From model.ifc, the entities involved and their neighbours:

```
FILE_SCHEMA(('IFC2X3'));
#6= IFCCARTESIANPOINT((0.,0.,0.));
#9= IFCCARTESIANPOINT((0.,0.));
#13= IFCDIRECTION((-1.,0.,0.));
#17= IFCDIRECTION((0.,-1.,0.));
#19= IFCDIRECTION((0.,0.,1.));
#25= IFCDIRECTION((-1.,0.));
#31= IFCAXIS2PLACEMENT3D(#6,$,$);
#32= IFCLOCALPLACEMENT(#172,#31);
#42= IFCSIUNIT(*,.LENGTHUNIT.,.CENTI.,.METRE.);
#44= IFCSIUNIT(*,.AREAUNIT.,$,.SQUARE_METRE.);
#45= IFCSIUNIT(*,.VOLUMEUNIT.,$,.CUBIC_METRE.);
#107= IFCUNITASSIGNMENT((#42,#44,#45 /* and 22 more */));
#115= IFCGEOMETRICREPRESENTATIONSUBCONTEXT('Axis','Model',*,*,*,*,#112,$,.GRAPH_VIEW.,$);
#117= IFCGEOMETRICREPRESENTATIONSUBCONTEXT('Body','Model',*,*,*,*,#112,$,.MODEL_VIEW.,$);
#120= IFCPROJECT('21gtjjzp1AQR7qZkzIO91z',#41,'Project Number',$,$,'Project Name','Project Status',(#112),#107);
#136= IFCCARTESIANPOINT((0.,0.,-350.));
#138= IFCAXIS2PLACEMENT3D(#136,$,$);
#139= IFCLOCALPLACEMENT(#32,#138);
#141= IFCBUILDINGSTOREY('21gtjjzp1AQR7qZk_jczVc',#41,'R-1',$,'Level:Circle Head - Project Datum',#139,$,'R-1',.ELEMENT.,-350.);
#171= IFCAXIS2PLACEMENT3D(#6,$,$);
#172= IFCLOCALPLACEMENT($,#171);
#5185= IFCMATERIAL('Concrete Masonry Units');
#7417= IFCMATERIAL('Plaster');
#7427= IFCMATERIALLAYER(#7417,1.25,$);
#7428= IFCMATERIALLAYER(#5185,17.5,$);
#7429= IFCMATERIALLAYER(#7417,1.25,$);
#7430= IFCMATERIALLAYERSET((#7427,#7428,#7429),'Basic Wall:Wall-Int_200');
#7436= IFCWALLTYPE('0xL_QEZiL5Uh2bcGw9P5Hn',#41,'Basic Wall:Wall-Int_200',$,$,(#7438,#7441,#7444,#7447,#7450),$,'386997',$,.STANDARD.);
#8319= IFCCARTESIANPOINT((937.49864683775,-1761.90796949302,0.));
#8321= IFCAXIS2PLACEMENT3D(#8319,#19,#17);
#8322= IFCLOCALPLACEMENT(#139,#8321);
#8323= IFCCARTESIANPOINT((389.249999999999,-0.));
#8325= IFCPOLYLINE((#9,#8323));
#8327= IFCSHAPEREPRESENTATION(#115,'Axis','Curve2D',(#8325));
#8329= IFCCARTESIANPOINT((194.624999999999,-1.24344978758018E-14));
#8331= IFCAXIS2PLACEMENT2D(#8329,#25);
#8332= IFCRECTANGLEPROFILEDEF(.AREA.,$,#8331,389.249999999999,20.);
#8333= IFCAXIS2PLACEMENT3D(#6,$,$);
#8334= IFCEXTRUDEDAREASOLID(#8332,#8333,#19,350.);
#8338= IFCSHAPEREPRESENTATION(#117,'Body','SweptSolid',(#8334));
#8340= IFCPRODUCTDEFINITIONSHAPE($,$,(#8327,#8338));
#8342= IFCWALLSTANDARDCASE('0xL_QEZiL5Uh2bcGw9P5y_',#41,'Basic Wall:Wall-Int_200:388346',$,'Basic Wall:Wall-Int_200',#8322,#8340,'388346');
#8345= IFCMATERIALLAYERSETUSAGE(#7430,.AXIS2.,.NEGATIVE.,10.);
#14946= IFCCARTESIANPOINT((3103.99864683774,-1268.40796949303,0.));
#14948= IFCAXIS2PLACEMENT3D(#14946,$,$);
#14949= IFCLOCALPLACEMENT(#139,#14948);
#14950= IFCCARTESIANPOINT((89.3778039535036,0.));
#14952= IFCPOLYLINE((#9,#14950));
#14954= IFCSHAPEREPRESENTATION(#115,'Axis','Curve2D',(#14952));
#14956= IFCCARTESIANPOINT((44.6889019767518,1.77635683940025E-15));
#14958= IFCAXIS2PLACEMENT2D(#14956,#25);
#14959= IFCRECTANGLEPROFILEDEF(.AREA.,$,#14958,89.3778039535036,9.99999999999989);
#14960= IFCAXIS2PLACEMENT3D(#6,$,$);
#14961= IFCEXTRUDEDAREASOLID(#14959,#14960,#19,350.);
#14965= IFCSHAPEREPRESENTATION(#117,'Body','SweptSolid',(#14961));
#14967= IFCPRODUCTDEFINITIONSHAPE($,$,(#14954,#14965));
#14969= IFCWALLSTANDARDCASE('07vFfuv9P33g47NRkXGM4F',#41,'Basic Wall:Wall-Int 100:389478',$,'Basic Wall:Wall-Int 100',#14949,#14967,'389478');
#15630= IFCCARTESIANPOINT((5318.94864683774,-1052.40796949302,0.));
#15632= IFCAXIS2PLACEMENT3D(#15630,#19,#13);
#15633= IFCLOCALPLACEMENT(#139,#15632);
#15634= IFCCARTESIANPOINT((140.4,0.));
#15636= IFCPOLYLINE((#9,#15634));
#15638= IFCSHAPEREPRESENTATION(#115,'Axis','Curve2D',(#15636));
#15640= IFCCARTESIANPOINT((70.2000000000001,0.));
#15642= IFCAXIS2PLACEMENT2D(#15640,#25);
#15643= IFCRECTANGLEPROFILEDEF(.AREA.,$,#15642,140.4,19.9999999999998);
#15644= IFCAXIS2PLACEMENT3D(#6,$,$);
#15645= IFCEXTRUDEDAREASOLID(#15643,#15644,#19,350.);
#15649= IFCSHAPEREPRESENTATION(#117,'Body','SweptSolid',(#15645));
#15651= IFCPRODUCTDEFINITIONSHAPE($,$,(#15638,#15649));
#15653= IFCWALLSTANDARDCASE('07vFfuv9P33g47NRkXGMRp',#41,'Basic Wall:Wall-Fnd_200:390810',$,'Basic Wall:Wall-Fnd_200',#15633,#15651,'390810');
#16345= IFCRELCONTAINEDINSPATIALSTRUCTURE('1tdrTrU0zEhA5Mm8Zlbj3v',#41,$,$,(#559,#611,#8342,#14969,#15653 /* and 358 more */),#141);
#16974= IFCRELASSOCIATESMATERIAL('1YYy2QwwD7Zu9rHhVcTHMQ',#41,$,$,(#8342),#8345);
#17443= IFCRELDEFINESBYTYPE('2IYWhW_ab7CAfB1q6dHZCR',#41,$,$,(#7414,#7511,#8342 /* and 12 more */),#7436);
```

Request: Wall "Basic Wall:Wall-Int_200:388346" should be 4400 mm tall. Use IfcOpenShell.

```python
import ifcopenshell
import ifcopenshell.geom
import ifcopenshell.util.representation
import ifcopenshell.util.shape
import ifcopenshell.util.unit

model = ifcopenshell.open("model.ifc")
unit_scale = ifcopenshell.util.unit.calculate_unit_scale(model)
settings = ifcopenshell.geom.settings()


def volume(element):
    """Net volume in cubic metres, openings subtracted."""
    shape = ifcopenshell.geom.create_shape(settings, element)
    return ifcopenshell.util.shape.get_volume(shape.geometry)


wall = model.by_guid("0xL_QEZiL5Uh2bcGw9P5y_")
before = volume(wall)

body = ifcopenshell.util.representation.get_representation(wall, "Model", "Body")
solid = body.Items[0]
old_height = solid.Depth
solid.Depth = 4.4 / unit_scale
after = volume(wall)

print(f"height {old_height:g} -> {solid.Depth:g}, volume {before:.3f} -> {after:.3f} m3")

model.write("model_updated.ifc")
```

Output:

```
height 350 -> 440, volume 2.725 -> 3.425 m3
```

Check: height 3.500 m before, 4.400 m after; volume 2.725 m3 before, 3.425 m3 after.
